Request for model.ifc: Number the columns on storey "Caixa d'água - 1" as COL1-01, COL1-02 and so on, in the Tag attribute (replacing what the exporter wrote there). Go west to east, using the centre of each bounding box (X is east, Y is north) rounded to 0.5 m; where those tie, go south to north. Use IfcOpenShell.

First a look at what the model holds.

```python
import ifcopenshell
import ifcopenshell.util.element
import ifcopenshell.util.placement

model = ifcopenshell.open("model.ifc")
print(model.schema)
storey = next(s for s in model.by_type("IfcBuildingStorey") if s.Name == "Caixa d'água - 1")
columns = [e for e in ifcopenshell.util.element.get_decomposition(storey) if e.is_a("IfcColumn")]
for e in sorted(columns, key=lambda e: e.id()):
    origin = ifcopenshell.util.placement.get_local_placement(e.ObjectPlacement)[:3, 3]
    print(e.id(), e.Tag, e.Name, origin.round(2) + 0.0, sep=" | ")
```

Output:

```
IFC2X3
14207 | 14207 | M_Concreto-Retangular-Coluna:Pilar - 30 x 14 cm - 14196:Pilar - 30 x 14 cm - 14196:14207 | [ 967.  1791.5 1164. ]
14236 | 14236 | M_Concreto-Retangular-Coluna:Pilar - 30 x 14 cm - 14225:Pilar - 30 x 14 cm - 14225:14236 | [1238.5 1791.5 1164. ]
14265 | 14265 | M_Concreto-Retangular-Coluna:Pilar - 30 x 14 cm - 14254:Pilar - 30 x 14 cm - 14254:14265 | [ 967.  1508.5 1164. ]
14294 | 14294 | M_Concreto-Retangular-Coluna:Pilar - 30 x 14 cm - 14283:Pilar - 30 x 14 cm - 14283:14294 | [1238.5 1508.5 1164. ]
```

```python
import ifcopenshell
import ifcopenshell.geom
import ifcopenshell.util.element
import ifcopenshell.util.shape

model = ifcopenshell.open("model.ifc")
settings = ifcopenshell.geom.settings()
settings.set("use-world-coords", True)


def centre(element):
    shape = ifcopenshell.geom.create_shape(settings, element)
    return ifcopenshell.util.shape.get_bbox_centroid(shape.geometry)


storey = next(s for s in model.by_type("IfcBuildingStorey") if s.Name == "Caixa d'água - 1")
columns = [e for e in ifcopenshell.util.element.get_decomposition(storey) if e.is_a("IfcColumn")]

# Insertion points can sit at a corner or the storey origin, so sort by the geometry (in metres).
centres = {e: centre(e) for e in columns}
columns.sort(key=lambda e: (round(centres[e][0] / 0.5), centres[e][1]))

for i, e in enumerate(columns, start=1):
    number = f"COL1-{i:02d}"
    e.Tag = number
    print(e.id(), number)

model.write("model_edited.ifc")
```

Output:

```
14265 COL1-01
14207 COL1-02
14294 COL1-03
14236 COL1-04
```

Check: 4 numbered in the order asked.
